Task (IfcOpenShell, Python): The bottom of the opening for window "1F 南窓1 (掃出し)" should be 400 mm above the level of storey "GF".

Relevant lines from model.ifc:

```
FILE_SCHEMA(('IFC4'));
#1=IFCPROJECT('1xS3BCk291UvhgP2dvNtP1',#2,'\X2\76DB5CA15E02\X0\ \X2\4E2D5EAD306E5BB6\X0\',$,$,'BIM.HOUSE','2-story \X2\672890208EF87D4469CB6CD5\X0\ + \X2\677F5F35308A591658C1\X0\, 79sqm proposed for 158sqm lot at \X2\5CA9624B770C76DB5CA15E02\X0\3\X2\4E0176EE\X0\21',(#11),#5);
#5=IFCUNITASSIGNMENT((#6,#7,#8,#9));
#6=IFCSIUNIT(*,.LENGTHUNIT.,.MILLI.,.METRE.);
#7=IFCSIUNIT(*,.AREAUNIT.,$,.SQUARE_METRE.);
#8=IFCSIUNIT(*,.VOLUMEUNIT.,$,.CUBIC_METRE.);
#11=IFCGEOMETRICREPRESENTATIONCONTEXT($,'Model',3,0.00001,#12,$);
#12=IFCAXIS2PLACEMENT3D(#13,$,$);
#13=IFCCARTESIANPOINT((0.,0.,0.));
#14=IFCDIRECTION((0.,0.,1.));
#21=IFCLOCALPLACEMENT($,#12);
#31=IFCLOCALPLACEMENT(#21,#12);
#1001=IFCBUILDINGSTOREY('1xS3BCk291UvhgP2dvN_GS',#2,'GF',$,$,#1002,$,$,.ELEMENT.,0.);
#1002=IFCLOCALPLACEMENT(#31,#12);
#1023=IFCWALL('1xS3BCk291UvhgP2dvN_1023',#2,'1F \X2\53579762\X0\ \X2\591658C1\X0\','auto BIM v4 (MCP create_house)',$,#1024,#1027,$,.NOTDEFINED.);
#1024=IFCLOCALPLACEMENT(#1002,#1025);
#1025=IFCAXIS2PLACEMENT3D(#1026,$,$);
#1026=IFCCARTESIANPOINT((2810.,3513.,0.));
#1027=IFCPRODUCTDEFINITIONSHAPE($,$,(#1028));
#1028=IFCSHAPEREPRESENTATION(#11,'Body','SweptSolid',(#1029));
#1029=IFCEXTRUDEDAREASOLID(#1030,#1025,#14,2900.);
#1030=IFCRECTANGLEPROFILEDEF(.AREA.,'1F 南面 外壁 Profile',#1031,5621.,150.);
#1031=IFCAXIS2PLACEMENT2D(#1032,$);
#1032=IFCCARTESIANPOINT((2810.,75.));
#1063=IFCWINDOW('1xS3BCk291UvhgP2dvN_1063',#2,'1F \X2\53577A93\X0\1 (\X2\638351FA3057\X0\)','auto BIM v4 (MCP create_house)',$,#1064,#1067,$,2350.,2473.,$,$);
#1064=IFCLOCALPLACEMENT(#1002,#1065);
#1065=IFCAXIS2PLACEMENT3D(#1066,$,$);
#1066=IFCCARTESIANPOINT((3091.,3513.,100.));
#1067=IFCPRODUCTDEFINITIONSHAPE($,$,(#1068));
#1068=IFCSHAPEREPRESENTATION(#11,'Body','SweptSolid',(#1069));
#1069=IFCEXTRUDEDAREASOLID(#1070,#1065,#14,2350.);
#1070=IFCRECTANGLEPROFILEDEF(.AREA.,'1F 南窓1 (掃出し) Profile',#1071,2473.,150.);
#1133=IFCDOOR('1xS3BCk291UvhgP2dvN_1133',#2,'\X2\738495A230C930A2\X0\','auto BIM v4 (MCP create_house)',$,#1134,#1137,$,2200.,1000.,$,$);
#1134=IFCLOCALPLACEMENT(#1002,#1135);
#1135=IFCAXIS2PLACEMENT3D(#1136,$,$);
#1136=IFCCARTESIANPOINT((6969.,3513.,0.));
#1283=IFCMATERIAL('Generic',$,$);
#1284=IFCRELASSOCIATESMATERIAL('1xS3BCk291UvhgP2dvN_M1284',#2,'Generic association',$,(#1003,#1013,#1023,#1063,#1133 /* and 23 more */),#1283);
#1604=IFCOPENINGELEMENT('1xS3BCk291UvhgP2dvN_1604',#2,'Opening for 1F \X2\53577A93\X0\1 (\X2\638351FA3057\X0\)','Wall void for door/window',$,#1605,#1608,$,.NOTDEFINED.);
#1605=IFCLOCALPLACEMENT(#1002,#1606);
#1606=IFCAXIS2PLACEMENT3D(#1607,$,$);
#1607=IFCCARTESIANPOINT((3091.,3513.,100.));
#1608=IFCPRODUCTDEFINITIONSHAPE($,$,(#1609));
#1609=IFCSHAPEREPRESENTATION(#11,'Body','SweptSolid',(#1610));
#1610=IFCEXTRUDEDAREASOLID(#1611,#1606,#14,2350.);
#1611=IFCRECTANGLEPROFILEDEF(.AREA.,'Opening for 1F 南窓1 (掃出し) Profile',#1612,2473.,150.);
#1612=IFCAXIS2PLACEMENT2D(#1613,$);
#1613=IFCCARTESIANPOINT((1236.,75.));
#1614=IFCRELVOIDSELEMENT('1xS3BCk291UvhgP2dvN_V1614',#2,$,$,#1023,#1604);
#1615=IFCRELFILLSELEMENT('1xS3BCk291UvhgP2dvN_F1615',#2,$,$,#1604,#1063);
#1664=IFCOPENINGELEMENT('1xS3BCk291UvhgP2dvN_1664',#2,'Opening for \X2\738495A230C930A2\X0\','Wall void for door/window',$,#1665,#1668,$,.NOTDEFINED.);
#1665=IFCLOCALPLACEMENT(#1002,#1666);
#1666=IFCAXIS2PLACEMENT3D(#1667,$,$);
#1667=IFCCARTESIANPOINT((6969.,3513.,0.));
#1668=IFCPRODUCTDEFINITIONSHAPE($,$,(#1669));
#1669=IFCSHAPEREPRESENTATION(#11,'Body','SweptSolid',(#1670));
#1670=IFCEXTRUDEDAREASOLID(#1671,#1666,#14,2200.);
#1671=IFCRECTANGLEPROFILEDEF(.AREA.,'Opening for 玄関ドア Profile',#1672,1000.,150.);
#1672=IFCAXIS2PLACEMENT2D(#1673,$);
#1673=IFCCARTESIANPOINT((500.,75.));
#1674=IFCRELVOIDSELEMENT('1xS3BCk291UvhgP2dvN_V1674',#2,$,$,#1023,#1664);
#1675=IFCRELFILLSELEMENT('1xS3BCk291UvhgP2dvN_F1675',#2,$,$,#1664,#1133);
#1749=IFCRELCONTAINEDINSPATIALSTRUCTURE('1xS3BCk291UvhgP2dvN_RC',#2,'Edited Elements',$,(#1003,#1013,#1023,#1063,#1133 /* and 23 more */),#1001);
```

```python
import numpy as np
import ifcopenshell
import ifcopenshell.api.geometry
import ifcopenshell.geom
import ifcopenshell.util.element
import ifcopenshell.util.placement
import ifcopenshell.util.shape
import ifcopenshell.util.unit

model = ifcopenshell.open("model.ifc")
unit_scale = ifcopenshell.util.unit.calculate_unit_scale(model)

window = model.by_guid("1xS3BCk291UvhgP2dvN_1063")
opening = window.FillsVoids[0].RelatingOpeningElement
storey = ifcopenshell.util.element.get_container(window, ifc_class="IfcBuildingStorey")
level = ifcopenshell.util.placement.get_local_placement(storey.ObjectPlacement)[2, 3]

# The opening's origin need not be at the sill, so measure its lowest point.
shape = ifcopenshell.geom.create_shape(ifcopenshell.geom.settings(), opening)
bottom = ifcopenshell.util.shape.get_shape_bottom_elevation(shape, shape.geometry) / unit_scale
dz = level + 400.0 - bottom

shift = np.array([0.0, 0.0, dz])
# The window is not placed relative to its opening, so move both.
for product in (opening, window):
    matrix = ifcopenshell.util.placement.get_local_placement(product.ObjectPlacement)
    matrix[:3, 3] += shift
    ifcopenshell.api.geometry.edit_object_placement(model, product=product, matrix=matrix, is_si=False)

print(f"moved by {dz * unit_scale:+.3f} m")

model.write("model-out.ifc")
```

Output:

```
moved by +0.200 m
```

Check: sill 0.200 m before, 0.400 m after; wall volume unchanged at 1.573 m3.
